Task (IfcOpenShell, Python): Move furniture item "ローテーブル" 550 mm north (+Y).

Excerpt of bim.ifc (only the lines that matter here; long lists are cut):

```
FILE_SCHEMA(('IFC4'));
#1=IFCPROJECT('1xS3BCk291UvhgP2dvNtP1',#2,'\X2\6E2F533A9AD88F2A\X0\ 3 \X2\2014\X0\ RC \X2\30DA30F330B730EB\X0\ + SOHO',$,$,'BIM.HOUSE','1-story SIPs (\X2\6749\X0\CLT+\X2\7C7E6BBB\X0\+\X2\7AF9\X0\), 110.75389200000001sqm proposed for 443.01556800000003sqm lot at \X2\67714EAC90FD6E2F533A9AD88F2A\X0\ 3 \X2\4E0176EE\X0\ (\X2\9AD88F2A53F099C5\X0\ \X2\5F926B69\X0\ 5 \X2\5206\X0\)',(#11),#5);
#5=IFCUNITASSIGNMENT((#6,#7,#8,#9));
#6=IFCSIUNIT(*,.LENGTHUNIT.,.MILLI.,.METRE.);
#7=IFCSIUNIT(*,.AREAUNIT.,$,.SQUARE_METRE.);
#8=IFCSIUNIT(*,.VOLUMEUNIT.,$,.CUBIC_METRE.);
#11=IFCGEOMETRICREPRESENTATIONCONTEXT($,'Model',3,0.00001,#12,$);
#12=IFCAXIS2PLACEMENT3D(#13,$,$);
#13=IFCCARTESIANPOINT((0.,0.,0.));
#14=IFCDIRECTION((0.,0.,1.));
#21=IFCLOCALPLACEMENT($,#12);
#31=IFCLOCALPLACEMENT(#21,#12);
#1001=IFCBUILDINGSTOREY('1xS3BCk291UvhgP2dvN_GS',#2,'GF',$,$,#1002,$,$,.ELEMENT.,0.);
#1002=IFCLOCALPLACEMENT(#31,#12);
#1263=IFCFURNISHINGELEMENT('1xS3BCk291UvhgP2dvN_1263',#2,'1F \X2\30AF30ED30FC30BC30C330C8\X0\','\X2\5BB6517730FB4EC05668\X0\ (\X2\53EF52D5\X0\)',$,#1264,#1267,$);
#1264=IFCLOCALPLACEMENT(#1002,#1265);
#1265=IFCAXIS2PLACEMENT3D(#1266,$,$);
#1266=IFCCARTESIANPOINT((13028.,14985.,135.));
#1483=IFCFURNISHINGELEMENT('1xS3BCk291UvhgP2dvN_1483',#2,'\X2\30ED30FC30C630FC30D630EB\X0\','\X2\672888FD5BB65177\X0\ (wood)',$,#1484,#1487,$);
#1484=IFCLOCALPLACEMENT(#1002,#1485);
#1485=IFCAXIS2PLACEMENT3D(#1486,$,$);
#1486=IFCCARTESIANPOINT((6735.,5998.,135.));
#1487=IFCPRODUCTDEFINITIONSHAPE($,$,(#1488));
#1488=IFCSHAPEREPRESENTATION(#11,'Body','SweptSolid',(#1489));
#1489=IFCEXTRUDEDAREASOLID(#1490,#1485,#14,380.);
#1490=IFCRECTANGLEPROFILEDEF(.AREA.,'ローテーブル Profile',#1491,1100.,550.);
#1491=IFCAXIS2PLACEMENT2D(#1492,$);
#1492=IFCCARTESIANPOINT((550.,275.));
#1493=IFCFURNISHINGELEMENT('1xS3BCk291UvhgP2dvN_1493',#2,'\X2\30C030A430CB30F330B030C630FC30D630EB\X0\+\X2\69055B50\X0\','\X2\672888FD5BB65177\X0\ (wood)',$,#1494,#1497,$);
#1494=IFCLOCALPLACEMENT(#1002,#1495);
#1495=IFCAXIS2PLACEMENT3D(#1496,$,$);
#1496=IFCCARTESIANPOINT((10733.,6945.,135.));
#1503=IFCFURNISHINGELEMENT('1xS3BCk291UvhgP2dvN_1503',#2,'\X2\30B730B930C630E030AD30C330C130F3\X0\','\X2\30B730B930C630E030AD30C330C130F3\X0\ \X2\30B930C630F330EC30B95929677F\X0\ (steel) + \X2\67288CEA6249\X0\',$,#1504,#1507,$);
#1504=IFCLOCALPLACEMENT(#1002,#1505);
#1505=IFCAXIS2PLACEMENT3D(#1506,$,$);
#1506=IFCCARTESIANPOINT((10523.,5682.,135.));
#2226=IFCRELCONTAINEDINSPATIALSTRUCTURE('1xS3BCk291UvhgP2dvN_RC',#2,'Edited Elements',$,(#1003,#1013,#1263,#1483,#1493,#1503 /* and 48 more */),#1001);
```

```python
import ifcopenshell
import ifcopenshell.api.geometry
import ifcopenshell.util.placement
import ifcopenshell.util.unit

model = ifcopenshell.open("bim.ifc")
unit_scale = ifcopenshell.util.unit.calculate_unit_scale(model)

item = model.by_guid("1xS3BCk291UvhgP2dvN_1483")
matrix = ifcopenshell.util.placement.get_local_placement(item.ObjectPlacement)
matrix[1, 3] += 0.55 / unit_scale
ifcopenshell.api.geometry.edit_object_placement(model, product=item, matrix=matrix, is_si=False)

print(ifcopenshell.util.placement.get_local_placement(item.ObjectPlacement).round(3) + 0.0)

model.write("bim_updated.ifc")
```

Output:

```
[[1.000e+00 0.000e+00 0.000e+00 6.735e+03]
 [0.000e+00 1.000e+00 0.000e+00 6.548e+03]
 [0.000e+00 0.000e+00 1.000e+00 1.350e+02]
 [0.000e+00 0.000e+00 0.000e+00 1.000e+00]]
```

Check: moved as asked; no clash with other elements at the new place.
